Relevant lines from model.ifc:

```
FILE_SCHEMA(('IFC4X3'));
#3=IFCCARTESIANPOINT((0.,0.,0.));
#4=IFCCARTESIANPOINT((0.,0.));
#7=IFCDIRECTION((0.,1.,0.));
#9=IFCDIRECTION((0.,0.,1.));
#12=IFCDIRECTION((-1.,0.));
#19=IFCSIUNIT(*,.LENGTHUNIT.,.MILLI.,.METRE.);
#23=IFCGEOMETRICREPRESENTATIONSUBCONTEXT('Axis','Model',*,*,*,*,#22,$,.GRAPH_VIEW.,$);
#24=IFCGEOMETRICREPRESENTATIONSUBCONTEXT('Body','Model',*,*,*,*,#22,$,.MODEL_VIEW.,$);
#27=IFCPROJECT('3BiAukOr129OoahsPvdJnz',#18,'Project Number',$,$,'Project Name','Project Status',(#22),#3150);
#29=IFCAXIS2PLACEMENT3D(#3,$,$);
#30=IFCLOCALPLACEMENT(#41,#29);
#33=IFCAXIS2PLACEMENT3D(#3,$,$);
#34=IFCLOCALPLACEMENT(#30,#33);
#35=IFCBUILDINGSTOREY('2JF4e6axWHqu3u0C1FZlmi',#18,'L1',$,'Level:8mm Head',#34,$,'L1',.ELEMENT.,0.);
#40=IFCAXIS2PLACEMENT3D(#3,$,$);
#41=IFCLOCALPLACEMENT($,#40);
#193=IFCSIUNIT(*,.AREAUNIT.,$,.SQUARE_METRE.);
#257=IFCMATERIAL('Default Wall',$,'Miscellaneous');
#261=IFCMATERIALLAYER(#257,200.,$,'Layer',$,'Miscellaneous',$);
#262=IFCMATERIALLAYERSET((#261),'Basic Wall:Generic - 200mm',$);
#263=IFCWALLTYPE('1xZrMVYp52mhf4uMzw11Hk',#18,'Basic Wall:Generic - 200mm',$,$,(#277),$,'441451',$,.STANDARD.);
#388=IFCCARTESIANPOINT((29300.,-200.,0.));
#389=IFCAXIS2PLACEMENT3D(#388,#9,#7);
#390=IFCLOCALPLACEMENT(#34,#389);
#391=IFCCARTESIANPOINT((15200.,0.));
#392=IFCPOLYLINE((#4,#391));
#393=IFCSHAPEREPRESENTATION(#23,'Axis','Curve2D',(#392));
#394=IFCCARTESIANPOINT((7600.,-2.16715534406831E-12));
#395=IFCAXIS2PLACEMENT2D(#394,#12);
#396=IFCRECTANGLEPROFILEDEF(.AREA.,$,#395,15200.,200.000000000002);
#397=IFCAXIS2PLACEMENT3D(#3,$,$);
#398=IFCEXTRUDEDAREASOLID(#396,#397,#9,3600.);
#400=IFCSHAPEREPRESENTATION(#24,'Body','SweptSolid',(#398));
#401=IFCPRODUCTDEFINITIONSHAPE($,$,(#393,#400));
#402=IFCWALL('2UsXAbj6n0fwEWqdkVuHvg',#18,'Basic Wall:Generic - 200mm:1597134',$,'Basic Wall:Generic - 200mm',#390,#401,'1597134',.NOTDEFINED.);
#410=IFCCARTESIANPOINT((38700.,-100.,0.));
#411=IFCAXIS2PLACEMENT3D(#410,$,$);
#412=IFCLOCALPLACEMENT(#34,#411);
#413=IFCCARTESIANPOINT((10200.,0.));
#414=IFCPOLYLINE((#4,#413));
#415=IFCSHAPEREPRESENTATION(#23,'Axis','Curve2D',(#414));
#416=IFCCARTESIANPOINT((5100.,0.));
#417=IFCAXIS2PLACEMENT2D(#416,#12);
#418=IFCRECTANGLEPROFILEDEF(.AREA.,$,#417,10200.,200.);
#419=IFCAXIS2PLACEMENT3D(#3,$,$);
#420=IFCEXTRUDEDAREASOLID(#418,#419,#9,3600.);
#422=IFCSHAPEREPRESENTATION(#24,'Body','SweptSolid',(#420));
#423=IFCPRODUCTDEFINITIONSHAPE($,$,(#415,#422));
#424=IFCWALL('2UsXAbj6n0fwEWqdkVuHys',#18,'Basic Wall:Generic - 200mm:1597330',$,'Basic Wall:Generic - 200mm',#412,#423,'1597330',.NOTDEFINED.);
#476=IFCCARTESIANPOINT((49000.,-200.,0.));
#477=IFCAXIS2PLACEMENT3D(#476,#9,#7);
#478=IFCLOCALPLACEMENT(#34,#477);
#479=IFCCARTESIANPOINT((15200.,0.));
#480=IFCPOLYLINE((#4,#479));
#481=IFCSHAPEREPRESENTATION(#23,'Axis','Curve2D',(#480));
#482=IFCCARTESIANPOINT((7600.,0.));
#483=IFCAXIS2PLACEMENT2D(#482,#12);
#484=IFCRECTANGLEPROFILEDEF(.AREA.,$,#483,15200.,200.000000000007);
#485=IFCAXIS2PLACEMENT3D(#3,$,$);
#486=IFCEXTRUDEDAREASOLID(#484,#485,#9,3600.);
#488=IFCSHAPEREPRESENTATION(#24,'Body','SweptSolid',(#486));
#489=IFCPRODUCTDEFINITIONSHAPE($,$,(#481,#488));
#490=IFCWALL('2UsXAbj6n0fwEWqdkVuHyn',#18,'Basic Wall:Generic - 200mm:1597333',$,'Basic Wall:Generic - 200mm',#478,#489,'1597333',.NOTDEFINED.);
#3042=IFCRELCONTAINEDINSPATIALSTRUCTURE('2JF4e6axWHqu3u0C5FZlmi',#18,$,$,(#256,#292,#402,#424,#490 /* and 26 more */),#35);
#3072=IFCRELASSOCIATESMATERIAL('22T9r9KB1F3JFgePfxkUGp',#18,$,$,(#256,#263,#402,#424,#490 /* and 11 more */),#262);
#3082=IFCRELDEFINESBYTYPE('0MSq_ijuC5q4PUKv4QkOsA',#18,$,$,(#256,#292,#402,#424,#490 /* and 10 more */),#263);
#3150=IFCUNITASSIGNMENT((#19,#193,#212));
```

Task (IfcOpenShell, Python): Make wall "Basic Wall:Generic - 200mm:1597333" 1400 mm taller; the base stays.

```python
import ifcopenshell
import ifcopenshell.geom
import ifcopenshell.util.representation
import ifcopenshell.util.shape
import ifcopenshell.util.unit

model = ifcopenshell.open("model.ifc")
unit_scale = ifcopenshell.util.unit.calculate_unit_scale(model)
settings = ifcopenshell.geom.settings()


def volume(element):
    """Net volume in cubic metres, openings subtracted."""
    shape = ifcopenshell.geom.create_shape(settings, element)
    return ifcopenshell.util.shape.get_volume(shape.geometry)


wall = model.by_guid("2UsXAbj6n0fwEWqdkVuHyn")
before = volume(wall)

body = ifcopenshell.util.representation.get_representation(wall, "Model", "Body")
solid = body.Items[0]
old_height = solid.Depth
solid.Depth += 1.4 / unit_scale
after = volume(wall)

print(f"height {old_height:g} -> {solid.Depth:g}, volume {before:.3f} -> {after:.3f} m3")

model.write("model_edited.ifc")
```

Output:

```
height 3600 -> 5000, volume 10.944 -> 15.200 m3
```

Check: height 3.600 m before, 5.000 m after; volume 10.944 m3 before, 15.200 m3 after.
